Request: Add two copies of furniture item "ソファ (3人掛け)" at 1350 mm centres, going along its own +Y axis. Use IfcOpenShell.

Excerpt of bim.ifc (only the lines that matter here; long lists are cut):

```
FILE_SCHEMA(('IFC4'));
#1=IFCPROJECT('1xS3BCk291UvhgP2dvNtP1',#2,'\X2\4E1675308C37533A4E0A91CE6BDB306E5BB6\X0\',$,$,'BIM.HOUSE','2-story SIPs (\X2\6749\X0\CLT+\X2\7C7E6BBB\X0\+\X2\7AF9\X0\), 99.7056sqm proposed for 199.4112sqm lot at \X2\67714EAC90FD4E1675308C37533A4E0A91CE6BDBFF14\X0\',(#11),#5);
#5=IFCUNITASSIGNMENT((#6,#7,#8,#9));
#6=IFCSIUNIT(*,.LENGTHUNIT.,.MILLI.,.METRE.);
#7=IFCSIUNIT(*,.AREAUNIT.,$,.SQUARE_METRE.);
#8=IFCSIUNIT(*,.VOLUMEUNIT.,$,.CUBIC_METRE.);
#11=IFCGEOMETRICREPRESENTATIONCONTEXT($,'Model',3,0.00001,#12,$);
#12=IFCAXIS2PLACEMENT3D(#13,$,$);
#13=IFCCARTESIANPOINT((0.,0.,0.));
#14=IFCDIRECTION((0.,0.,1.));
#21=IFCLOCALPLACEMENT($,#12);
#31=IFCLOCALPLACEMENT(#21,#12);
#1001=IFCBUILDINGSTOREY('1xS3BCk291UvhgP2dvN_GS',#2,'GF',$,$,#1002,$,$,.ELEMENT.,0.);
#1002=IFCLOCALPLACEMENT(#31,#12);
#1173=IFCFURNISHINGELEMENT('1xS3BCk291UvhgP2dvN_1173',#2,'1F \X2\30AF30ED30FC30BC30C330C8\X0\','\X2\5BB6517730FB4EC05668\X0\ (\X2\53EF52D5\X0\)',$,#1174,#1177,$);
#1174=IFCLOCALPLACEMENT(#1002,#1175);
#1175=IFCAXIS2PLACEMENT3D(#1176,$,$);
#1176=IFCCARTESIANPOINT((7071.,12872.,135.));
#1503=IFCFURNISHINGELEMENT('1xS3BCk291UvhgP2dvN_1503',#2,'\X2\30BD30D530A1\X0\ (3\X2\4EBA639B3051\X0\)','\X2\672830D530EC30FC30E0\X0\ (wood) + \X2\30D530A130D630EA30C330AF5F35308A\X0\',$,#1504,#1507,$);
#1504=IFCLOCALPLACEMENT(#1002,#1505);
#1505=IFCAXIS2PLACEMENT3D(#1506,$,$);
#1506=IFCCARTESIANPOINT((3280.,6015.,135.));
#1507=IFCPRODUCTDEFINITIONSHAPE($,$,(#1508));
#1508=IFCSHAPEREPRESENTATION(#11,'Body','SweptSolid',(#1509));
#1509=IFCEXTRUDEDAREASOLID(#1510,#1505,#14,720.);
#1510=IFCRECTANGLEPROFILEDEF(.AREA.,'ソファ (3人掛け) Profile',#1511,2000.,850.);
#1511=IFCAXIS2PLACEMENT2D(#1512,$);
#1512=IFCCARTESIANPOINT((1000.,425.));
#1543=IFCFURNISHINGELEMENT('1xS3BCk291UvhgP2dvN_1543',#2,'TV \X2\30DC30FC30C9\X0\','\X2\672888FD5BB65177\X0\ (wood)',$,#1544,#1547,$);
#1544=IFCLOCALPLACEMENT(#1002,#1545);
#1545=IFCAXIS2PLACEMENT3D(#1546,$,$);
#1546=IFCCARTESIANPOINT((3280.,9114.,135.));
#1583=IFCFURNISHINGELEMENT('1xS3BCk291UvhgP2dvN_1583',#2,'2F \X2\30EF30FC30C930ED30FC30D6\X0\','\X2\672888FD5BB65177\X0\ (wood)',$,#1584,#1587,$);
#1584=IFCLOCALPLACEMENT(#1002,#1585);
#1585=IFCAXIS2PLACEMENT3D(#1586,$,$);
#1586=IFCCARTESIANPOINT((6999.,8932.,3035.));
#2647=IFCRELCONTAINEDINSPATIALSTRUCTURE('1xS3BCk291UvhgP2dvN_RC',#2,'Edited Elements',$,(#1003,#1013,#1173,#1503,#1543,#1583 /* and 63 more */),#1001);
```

```python
import ifcopenshell
import ifcopenshell.api.geometry
import ifcopenshell.api.root
import ifcopenshell.util.element
import ifcopenshell.util.placement
import ifcopenshell.util.unit

model = ifcopenshell.open("bim.ifc")
unit_scale = ifcopenshell.util.unit.calculate_unit_scale(model)


def reuse_history(source, copy):
    """copy_class also copies each property set's owner history, people and application; keep the originals."""
    for rel in copy.IsDefinedBy:
        if rel.is_a("IfcRelDefinesByProperties") and (history := rel.RelatingPropertyDefinition.OwnerHistory):
            rel.RelatingPropertyDefinition.OwnerHistory = source.OwnerHistory
            ifcopenshell.util.element.remove_deep2(model, history)


source = model.by_guid("1xS3BCk291UvhgP2dvN_1503")
base = ifcopenshell.util.placement.get_local_placement(source.ObjectPlacement)
step = base[:3, 1] * 1.35 / unit_scale

for i in range(1, 3):
    copy = ifcopenshell.api.root.copy_class(model, product=source)
    copy.Representation = ifcopenshell.util.element.copy_deep(
        model, source.Representation, exclude=["IfcGeometricRepresentationContext", "IfcRepresentationMap"]
    )
    reuse_history(source, copy)
    matrix = base.copy()
    matrix[:3, 3] += i * step
    print("added at", matrix[:3, 3].round(3) + 0.0)
    ifcopenshell.api.geometry.edit_object_placement(model, product=copy, matrix=matrix, is_si=False)

model.write("bim_rev.ifc")
```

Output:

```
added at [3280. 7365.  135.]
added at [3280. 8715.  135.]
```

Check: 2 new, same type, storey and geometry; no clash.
